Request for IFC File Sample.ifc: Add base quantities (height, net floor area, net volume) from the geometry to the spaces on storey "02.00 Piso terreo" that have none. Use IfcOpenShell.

First a look at what the model holds.

```python
import ifcopenshell
import ifcopenshell.util.element
import ifcopenshell.util.unit

model = ifcopenshell.open("IFC File Sample.ifc")
print(model.schema)
for unit_type in ("LENGTHUNIT", "AREAUNIT", "VOLUMEUNIT"):
    print(unit_type, ifcopenshell.util.unit.calculate_unit_scale(model, unit_type))
storey = next(s for s in model.by_type("IfcBuildingStorey") if s.Name == "02.00 Piso terreo")
spaces = [e for e in ifcopenshell.util.element.get_decomposition(storey) if e.is_a("IfcSpace")]
for e in sorted(spaces, key=lambda e: e.id()):
    print(e.id(), e.is_a(), e.Name, list(ifcopenshell.util.element.get_psets(e, qtos_only=True)), sep=" | ")
```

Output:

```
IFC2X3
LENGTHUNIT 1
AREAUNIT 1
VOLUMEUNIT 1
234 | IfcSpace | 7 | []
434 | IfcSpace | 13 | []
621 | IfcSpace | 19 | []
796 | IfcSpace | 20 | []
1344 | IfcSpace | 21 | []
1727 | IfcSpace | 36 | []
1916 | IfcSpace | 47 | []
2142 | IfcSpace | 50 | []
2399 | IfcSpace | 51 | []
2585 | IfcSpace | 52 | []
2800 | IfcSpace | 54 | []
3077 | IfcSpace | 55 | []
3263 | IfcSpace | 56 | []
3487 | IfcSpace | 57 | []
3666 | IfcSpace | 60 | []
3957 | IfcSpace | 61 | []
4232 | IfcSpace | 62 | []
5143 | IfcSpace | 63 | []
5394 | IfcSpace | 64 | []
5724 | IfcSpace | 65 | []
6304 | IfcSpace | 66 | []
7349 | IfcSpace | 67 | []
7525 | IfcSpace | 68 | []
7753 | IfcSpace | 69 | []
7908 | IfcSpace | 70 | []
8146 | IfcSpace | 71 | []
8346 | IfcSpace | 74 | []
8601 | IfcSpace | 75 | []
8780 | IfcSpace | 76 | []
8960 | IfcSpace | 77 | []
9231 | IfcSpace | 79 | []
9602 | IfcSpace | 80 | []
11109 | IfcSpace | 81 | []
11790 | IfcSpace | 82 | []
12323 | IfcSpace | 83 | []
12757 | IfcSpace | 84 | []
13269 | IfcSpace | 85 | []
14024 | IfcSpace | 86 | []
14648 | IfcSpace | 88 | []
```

```python
import ifcopenshell
import ifcopenshell.api.pset
import ifcopenshell.geom
import ifcopenshell.util.element
import ifcopenshell.util.shape
import ifcopenshell.util.unit

model = ifcopenshell.open("IFC File Sample.ifc")
unit_scale = ifcopenshell.util.unit.calculate_unit_scale(model)
area_scale = ifcopenshell.util.unit.calculate_unit_scale(model, "AREAUNIT")
volume_scale = ifcopenshell.util.unit.calculate_unit_scale(model, "VOLUMEUNIT")
settings = ifcopenshell.geom.settings()

storey = next(s for s in model.by_type("IfcBuildingStorey") if s.Name == "02.00 Piso terreo")
spaces = [e for e in ifcopenshell.util.element.get_decomposition(storey) if e.is_a("IfcSpace")]

for e in sorted(spaces, key=lambda e: e.id()):
    if ifcopenshell.util.element.get_psets(e, qtos_only=True, should_inherit=False):
        continue
    # Geometry comes back in metres, in the element's own axes.
    shape = ifcopenshell.geom.create_shape(settings, e)
    values = {
        "Height": ifcopenshell.util.shape.get_z(shape.geometry) / unit_scale,
        "NetFloorArea": ifcopenshell.util.shape.get_footprint_area(shape.geometry) / area_scale,
        "NetVolume": ifcopenshell.util.shape.get_volume(shape.geometry) / volume_scale,
    }
    qto = ifcopenshell.api.pset.add_qto(model, product=e, name="BaseQuantities")
    ifcopenshell.api.pset.edit_qto(model, qto=qto, properties=values)
    print(e.id(), {k: round(v, 3) for k, v in values.items()})

model.write("IFC File Sample_v2.ifc")
```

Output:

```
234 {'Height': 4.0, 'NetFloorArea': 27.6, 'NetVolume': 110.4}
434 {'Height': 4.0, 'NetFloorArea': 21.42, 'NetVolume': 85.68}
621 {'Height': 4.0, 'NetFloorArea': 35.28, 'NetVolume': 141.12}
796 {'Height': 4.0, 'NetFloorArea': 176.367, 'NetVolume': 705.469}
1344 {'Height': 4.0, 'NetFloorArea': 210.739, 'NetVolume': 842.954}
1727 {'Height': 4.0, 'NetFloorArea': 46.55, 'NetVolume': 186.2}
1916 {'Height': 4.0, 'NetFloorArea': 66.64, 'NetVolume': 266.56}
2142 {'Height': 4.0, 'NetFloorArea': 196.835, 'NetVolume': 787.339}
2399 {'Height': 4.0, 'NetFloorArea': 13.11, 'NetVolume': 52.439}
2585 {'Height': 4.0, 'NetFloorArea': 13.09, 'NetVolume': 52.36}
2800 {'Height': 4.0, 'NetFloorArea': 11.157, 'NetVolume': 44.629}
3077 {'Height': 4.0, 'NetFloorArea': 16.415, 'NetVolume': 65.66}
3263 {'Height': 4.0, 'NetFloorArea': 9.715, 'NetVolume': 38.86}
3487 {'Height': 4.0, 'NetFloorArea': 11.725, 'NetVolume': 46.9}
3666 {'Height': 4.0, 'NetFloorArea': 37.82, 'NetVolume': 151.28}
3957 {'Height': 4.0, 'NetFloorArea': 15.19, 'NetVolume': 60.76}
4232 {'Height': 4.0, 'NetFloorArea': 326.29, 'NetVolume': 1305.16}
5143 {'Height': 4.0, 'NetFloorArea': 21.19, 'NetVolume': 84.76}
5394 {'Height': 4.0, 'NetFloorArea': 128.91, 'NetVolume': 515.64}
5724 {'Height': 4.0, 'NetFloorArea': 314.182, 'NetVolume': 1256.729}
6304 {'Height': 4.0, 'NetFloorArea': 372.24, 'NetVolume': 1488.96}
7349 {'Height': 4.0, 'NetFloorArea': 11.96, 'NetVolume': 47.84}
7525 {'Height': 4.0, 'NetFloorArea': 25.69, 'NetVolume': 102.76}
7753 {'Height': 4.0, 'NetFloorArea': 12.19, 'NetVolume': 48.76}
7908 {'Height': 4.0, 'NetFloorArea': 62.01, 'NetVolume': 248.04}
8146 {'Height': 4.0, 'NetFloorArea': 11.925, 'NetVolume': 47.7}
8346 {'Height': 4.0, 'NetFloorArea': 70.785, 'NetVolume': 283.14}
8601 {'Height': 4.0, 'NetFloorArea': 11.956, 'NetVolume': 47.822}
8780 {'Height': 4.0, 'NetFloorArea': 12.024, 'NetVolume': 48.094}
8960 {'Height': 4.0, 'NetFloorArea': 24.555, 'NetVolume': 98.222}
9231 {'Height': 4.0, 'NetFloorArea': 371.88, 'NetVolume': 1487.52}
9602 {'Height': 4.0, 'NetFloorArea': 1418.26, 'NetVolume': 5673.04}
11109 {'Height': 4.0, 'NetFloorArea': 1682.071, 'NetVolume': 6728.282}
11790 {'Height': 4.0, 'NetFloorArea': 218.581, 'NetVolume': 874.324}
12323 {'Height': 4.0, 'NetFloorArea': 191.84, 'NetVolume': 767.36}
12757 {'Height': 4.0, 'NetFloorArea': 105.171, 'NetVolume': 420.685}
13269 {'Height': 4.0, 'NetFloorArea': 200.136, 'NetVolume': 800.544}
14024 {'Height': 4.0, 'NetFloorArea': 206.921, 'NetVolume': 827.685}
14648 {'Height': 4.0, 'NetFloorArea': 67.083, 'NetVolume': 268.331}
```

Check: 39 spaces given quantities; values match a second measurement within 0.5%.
